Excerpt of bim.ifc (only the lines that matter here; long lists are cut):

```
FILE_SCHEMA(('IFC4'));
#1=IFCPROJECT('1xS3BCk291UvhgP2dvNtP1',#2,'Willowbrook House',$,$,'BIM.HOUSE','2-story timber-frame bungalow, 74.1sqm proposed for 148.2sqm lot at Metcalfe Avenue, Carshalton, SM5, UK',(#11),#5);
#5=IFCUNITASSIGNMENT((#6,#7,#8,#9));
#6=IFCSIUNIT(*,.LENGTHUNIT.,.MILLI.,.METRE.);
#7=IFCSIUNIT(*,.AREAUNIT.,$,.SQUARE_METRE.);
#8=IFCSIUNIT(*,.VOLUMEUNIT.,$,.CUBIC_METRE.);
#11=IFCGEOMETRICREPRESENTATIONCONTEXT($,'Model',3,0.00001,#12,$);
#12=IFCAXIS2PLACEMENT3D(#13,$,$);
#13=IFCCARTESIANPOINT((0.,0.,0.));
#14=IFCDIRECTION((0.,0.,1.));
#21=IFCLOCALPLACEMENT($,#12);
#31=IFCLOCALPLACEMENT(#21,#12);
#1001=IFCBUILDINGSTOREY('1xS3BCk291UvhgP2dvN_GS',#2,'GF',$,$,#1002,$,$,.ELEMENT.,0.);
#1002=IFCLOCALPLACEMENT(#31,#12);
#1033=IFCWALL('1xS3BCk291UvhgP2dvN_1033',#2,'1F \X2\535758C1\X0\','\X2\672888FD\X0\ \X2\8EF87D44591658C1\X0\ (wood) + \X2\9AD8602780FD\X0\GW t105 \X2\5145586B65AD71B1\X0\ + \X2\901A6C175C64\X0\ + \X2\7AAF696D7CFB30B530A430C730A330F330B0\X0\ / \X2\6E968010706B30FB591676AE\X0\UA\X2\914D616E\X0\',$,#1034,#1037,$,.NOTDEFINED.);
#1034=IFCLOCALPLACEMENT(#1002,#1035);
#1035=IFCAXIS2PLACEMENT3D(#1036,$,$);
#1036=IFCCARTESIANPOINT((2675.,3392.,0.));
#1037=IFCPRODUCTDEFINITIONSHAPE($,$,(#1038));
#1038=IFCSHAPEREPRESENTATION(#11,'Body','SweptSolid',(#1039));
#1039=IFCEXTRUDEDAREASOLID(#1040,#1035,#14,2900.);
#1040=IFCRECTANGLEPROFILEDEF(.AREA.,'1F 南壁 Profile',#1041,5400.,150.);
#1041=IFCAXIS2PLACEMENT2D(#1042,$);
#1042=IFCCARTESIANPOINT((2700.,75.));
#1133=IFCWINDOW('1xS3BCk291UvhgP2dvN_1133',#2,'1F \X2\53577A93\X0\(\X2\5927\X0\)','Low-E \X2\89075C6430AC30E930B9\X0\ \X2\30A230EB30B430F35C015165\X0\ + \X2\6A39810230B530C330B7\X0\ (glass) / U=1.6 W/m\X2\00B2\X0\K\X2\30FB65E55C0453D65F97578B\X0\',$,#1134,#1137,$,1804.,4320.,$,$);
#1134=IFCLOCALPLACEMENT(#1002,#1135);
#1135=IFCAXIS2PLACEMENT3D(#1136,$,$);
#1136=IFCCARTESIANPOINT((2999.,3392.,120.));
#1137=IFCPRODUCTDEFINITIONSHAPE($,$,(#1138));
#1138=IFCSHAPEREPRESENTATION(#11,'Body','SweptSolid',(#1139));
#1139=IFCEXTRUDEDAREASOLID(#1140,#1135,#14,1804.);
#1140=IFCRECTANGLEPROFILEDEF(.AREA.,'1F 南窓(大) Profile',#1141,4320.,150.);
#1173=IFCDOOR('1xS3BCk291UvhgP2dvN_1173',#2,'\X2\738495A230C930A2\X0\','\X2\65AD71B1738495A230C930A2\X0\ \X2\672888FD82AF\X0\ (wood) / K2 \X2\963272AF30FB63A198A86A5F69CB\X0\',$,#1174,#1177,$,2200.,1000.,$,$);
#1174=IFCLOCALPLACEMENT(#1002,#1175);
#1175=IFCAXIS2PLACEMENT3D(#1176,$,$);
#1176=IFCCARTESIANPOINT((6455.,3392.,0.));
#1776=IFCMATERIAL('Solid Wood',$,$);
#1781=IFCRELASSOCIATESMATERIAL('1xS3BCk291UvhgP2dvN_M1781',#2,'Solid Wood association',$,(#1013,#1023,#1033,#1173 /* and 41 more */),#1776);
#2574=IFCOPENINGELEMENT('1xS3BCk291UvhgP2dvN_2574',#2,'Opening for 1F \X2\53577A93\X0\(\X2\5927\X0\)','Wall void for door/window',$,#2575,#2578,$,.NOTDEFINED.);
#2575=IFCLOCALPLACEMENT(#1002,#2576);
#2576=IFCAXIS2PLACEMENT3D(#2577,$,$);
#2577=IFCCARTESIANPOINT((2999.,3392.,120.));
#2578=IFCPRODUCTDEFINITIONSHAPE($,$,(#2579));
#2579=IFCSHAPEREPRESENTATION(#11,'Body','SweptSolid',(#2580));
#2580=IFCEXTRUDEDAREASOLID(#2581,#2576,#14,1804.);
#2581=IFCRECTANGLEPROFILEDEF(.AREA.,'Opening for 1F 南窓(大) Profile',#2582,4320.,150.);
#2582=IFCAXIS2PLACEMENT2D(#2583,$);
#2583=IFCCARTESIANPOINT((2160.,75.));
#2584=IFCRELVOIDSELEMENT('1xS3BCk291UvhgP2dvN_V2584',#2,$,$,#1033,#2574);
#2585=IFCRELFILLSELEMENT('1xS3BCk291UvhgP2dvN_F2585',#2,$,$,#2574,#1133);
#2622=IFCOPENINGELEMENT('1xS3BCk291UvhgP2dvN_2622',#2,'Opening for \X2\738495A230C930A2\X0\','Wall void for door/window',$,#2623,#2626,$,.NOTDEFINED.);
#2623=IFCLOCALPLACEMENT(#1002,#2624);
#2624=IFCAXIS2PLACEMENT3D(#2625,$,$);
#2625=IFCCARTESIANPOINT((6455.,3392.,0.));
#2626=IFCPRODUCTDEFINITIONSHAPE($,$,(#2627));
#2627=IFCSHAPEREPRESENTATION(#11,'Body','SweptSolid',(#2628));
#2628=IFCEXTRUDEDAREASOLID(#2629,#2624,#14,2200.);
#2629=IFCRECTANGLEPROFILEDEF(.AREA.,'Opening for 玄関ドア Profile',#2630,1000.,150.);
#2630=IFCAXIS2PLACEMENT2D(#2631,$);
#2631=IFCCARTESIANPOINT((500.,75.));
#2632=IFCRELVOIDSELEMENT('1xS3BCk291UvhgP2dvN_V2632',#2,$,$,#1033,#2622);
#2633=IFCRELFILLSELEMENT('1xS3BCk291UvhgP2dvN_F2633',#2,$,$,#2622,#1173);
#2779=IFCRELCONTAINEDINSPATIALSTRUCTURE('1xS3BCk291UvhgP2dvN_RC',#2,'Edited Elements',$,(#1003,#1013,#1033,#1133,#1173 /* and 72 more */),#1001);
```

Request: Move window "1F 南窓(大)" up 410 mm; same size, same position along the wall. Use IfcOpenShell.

```python
import numpy as np
import ifcopenshell
import ifcopenshell.api.geometry
import ifcopenshell.util.placement
import ifcopenshell.util.unit

model = ifcopenshell.open("bim.ifc")
unit_scale = ifcopenshell.util.unit.calculate_unit_scale(model)

window = model.by_guid("1xS3BCk291UvhgP2dvN_1133")
opening = window.FillsVoids[0].RelatingOpeningElement
dz = 410.0

shift = np.array([0.0, 0.0, dz])
# The window is not placed relative to its opening, so move both.
for product in (opening, window):
    matrix = ifcopenshell.util.placement.get_local_placement(product.ObjectPlacement)
    matrix[:3, 3] += shift
    ifcopenshell.api.geometry.edit_object_placement(model, product=product, matrix=matrix, is_si=False)

print(f"moved by {dz * unit_scale:+.3f} m")

model.write("bim_v2.ifc")
```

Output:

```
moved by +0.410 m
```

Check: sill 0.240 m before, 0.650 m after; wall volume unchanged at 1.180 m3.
